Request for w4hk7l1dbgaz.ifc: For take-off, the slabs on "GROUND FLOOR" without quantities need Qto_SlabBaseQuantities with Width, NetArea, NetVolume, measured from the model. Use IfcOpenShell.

First a look at what the model holds.

```python
import ifcopenshell
import ifcopenshell.util.element
import ifcopenshell.util.unit

model = ifcopenshell.open("w4hk7l1dbgaz.ifc")
print(model.schema)
for unit_type in ("LENGTHUNIT", "AREAUNIT", "VOLUMEUNIT"):
    print(unit_type, ifcopenshell.util.unit.calculate_unit_scale(model, unit_type))
storey = next(s for s in model.by_type("IfcBuildingStorey") if s.Name == "GROUND FLOOR")
slabs = [e for e in ifcopenshell.util.element.get_decomposition(storey) if e.is_a("IfcSlab")]
for e in sorted(slabs, key=lambda e: e.id()):
    print(e.id(), e.is_a(), e.Name, list(ifcopenshell.util.element.get_psets(e, qtos_only=True)), sep=" | ")
```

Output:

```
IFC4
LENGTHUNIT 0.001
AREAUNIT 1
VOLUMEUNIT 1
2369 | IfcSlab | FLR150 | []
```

```python
import ifcopenshell
import ifcopenshell.api.pset
import ifcopenshell.geom
import ifcopenshell.util.element
import ifcopenshell.util.shape
import ifcopenshell.util.unit

model = ifcopenshell.open("w4hk7l1dbgaz.ifc")
unit_scale = ifcopenshell.util.unit.calculate_unit_scale(model)
area_scale = ifcopenshell.util.unit.calculate_unit_scale(model, "AREAUNIT")
volume_scale = ifcopenshell.util.unit.calculate_unit_scale(model, "VOLUMEUNIT")
settings = ifcopenshell.geom.settings()

storey = next(s for s in model.by_type("IfcBuildingStorey") if s.Name == "GROUND FLOOR")
slabs = [e for e in ifcopenshell.util.element.get_decomposition(storey) if e.is_a("IfcSlab")]

for e in sorted(slabs, key=lambda e: e.id()):
    if ifcopenshell.util.element.get_psets(e, qtos_only=True, should_inherit=False):
        continue
    # Geometry comes back in metres, in the element's own axes.
    shape = ifcopenshell.geom.create_shape(settings, e)
    values = {
        "Width": ifcopenshell.util.shape.get_z(shape.geometry) / unit_scale,
        "NetArea": ifcopenshell.util.shape.get_footprint_area(shape.geometry) / area_scale,
        "NetVolume": ifcopenshell.util.shape.get_volume(shape.geometry) / volume_scale,
    }
    qto = ifcopenshell.api.pset.add_qto(model, product=e, name="Qto_SlabBaseQuantities")
    ifcopenshell.api.pset.edit_qto(model, qto=qto, properties=values)
    print(e.id(), {k: round(v, 3) for k, v in values.items()})

model.write("w4hk7l1dbgaz_updated.ifc")
```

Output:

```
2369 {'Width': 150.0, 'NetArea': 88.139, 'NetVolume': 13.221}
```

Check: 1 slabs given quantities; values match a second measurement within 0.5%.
